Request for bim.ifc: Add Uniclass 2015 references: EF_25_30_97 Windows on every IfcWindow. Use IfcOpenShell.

First a look at what the model holds.

```python
import ifcopenshell

model = ifcopenshell.open("bim.ifc")
print(model.schema)
print("classifications:", [c.Name for c in model.by_type("IfcClassification")])
for ifc_class in ("IfcDoor", "IfcRoof", "IfcStair", "IfcWall", "IfcWindow"):
    print(ifc_class, len(model.by_type(ifc_class)))
```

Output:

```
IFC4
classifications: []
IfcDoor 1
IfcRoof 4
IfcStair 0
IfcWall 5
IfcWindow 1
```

```python
import ifcopenshell
import ifcopenshell.api.classification

model = ifcopenshell.open("bim.ifc")

system = ifcopenshell.api.classification.add_classification(model, classification="Uniclass 2015")

codes = {
    "IfcWindow": ("EF_25_30_97", "Windows"),
}
for ifc_class, (code, name) in codes.items():
    products = model.by_type(ifc_class)
    ifcopenshell.api.classification.add_reference(
        model, products=products, classification=system, identification=code, name=name
    )
    print(code, len(products))

model.write("bim_updated.ifc")
```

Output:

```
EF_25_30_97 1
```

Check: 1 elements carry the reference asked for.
